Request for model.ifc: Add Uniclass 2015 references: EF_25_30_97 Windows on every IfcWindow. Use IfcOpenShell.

First a look at what the model holds.

```python
import ifcopenshell

model = ifcopenshell.open("model.ifc")
print(model.schema)
print("classifications:", [c.Name for c in model.by_type("IfcClassification")])
for ifc_class in ("IfcDoor", "IfcRoof", "IfcStair", "IfcWall", "IfcWindow"):
    print(ifc_class, len(model.by_type(ifc_class)))
```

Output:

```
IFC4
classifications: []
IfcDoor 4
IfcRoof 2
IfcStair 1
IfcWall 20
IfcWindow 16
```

```python
import ifcopenshell
import ifcopenshell.api.classification

model = ifcopenshell.open("model.ifc")

system = ifcopenshell.api.classification.add_classification(model, classification="Uniclass 2015")

codes = {
    "IfcWindow": ("EF_25_30_97", "Windows"),
}
for ifc_class, (code, name) in codes.items():
    products = model.by_type(ifc_class)
    ifcopenshell.api.classification.add_reference(
        model, products=products, classification=system, identification=code, name=name
    )
    print(code, len(products))

model.write("model_updated.ifc")
```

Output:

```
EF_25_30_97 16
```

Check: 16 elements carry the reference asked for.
